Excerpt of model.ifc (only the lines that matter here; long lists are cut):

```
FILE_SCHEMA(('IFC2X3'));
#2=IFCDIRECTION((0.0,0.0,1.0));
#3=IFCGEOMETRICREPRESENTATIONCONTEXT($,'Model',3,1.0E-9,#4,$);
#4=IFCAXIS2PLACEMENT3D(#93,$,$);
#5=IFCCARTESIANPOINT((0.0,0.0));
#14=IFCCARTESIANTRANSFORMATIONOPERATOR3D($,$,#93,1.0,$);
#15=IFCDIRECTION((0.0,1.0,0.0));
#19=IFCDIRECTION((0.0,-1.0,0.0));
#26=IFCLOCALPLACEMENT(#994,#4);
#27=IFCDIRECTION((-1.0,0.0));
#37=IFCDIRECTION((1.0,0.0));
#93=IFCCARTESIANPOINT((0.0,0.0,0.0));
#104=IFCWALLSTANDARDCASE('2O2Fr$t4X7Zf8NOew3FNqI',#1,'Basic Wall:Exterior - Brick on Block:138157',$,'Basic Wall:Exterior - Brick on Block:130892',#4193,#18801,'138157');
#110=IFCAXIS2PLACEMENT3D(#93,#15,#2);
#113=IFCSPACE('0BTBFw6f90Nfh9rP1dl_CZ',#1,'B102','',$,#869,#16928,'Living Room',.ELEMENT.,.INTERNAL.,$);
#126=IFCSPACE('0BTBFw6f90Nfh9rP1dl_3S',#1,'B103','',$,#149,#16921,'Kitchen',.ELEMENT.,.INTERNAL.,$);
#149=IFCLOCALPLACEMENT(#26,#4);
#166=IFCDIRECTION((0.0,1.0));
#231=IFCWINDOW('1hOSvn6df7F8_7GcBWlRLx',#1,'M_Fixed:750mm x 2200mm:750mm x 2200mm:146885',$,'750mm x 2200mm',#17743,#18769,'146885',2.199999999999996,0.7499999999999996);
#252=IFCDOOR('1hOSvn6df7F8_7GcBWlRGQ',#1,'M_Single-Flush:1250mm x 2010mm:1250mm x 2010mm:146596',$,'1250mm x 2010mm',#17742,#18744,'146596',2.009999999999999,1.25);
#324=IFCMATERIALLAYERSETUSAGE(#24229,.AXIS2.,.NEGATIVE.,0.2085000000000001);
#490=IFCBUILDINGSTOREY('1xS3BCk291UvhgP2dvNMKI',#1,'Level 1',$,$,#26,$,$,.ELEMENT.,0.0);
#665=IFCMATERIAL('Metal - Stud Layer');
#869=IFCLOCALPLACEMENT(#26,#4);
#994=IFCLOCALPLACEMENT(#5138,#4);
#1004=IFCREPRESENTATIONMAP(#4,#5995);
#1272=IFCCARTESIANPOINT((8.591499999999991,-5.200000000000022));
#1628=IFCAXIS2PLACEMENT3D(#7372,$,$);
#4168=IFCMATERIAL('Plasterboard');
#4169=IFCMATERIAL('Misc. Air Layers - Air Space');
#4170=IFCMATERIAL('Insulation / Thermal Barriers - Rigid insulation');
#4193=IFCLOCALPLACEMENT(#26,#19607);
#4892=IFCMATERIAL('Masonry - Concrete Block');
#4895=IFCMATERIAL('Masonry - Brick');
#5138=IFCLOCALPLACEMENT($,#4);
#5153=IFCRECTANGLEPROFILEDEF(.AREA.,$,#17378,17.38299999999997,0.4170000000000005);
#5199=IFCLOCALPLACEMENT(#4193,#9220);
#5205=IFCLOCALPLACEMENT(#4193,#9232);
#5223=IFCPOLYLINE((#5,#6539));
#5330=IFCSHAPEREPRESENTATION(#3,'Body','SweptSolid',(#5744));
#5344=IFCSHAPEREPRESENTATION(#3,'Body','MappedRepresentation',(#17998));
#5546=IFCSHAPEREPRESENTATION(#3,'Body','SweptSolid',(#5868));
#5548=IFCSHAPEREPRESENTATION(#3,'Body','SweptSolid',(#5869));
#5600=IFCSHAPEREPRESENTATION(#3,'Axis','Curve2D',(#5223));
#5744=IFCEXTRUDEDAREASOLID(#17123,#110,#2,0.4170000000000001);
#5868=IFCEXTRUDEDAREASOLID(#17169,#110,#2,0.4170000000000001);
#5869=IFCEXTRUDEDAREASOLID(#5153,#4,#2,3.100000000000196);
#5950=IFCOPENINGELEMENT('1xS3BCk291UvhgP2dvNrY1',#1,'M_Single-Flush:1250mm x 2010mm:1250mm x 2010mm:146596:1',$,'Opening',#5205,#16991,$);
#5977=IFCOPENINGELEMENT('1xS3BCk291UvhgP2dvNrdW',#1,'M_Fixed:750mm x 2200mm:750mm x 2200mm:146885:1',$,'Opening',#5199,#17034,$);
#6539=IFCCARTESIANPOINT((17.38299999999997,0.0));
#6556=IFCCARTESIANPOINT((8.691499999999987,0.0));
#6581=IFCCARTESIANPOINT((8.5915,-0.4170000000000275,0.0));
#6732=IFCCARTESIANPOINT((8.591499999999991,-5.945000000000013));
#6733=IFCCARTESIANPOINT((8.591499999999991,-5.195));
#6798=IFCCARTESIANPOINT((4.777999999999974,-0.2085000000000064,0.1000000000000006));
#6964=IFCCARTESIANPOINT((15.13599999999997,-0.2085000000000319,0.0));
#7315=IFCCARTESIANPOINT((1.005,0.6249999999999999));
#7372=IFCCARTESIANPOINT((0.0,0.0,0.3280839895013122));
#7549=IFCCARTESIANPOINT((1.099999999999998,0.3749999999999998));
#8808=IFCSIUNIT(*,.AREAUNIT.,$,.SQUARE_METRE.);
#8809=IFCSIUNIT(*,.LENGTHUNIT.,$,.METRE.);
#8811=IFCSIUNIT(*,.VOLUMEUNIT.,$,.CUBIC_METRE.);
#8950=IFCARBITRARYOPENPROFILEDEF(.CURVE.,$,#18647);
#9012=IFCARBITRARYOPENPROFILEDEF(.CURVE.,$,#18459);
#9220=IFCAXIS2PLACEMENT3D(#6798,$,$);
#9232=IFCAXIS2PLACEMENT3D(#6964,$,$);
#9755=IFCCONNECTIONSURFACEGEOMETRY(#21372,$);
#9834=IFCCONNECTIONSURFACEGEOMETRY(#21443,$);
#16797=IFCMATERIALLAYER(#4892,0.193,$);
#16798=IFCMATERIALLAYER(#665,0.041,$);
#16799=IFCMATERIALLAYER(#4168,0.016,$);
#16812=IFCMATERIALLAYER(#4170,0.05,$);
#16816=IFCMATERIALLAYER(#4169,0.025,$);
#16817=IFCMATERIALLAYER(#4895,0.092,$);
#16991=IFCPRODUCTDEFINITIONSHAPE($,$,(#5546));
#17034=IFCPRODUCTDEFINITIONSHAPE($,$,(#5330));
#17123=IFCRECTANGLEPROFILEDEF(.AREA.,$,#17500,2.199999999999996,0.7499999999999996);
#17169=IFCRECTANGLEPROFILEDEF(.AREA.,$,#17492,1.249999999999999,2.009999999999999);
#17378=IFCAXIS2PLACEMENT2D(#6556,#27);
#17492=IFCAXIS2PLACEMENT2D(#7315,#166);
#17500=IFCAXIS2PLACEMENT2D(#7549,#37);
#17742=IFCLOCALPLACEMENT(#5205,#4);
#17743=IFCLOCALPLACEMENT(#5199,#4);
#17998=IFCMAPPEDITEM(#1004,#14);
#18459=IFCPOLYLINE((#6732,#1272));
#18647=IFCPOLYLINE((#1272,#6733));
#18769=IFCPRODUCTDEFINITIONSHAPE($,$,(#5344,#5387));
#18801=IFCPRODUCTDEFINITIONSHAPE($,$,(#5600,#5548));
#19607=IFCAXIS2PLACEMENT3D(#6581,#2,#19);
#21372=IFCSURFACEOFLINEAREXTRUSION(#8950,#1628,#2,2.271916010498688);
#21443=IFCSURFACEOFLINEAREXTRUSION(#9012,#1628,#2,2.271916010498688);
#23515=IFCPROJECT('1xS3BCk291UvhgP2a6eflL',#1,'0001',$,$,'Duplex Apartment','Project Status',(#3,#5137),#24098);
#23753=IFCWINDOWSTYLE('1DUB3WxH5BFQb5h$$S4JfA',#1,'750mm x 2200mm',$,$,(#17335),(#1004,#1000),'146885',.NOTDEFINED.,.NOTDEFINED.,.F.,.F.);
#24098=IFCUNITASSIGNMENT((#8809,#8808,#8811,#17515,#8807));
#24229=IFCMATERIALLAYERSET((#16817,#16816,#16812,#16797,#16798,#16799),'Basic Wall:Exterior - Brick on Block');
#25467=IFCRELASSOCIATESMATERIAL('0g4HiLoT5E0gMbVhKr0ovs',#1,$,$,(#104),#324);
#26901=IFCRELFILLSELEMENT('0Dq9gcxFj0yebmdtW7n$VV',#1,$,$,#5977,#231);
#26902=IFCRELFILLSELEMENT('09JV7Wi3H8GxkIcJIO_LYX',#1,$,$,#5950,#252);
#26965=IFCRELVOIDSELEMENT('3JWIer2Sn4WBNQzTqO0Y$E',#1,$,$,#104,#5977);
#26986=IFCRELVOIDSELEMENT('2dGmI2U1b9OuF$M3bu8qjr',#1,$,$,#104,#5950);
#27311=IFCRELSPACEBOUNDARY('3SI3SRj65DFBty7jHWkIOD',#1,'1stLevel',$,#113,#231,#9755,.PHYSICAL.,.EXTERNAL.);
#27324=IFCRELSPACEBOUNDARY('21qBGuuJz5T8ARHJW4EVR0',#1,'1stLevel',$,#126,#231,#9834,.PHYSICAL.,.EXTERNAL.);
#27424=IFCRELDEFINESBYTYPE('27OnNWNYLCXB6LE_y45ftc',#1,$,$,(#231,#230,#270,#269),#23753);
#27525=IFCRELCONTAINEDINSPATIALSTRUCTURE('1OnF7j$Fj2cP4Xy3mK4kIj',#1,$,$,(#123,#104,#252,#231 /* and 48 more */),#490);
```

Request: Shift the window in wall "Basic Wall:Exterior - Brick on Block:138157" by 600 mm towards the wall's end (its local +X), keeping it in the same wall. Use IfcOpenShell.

```python
import numpy as np
import ifcopenshell
import ifcopenshell.api.geometry
import ifcopenshell.util.placement

model = ifcopenshell.open("model.ifc")

window = model.by_guid("1hOSvn6df7F8_7GcBWlRLx")
opening = window.FillsVoids[0].RelatingOpeningElement
wall = opening.VoidsElements[0].RelatingBuildingElement

wall_matrix = ifcopenshell.util.placement.get_local_placement(wall.ObjectPlacement)
shift = wall_matrix[:3, 0] * 0.6
before = ifcopenshell.util.placement.get_local_placement(window.ObjectPlacement)[:3, 3].copy()

# The window is placed relative to its opening, so it follows when the opening moves.
matrix = ifcopenshell.util.placement.get_local_placement(opening.ObjectPlacement)
matrix[:3, 3] += shift
ifcopenshell.api.geometry.edit_object_placement(
    model, product=opening, matrix=matrix, is_si=False, should_transform_children=True
)

# Space boundary surfaces are stored in each space's coordinates; move them too.
for rel in window.ProvidesBoundaries:
    if not rel.ConnectionGeometry:
        continue
    surface = rel.ConnectionGeometry.SurfaceOnRelatingElement
    space_matrix = ifcopenshell.util.placement.get_local_placement(rel.RelatingSpace.ObjectPlacement)
    point = np.array(surface.Position.Location.Coordinates) + space_matrix[:3, :3].T @ shift
    surface.Position = model.createIfcAxis2Placement3D(
        model.createIfcCartesianPoint(point.tolist()), surface.Position.Axis, surface.Position.RefDirection
    )

after = ifcopenshell.util.placement.get_local_placement(window.ObjectPlacement)[:3, 3]
print("window moved by", (after - before).round(3) + 0.0)

model.write("model_updated.ifc")
```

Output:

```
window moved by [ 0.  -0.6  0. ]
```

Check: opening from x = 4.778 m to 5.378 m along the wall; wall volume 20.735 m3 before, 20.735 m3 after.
